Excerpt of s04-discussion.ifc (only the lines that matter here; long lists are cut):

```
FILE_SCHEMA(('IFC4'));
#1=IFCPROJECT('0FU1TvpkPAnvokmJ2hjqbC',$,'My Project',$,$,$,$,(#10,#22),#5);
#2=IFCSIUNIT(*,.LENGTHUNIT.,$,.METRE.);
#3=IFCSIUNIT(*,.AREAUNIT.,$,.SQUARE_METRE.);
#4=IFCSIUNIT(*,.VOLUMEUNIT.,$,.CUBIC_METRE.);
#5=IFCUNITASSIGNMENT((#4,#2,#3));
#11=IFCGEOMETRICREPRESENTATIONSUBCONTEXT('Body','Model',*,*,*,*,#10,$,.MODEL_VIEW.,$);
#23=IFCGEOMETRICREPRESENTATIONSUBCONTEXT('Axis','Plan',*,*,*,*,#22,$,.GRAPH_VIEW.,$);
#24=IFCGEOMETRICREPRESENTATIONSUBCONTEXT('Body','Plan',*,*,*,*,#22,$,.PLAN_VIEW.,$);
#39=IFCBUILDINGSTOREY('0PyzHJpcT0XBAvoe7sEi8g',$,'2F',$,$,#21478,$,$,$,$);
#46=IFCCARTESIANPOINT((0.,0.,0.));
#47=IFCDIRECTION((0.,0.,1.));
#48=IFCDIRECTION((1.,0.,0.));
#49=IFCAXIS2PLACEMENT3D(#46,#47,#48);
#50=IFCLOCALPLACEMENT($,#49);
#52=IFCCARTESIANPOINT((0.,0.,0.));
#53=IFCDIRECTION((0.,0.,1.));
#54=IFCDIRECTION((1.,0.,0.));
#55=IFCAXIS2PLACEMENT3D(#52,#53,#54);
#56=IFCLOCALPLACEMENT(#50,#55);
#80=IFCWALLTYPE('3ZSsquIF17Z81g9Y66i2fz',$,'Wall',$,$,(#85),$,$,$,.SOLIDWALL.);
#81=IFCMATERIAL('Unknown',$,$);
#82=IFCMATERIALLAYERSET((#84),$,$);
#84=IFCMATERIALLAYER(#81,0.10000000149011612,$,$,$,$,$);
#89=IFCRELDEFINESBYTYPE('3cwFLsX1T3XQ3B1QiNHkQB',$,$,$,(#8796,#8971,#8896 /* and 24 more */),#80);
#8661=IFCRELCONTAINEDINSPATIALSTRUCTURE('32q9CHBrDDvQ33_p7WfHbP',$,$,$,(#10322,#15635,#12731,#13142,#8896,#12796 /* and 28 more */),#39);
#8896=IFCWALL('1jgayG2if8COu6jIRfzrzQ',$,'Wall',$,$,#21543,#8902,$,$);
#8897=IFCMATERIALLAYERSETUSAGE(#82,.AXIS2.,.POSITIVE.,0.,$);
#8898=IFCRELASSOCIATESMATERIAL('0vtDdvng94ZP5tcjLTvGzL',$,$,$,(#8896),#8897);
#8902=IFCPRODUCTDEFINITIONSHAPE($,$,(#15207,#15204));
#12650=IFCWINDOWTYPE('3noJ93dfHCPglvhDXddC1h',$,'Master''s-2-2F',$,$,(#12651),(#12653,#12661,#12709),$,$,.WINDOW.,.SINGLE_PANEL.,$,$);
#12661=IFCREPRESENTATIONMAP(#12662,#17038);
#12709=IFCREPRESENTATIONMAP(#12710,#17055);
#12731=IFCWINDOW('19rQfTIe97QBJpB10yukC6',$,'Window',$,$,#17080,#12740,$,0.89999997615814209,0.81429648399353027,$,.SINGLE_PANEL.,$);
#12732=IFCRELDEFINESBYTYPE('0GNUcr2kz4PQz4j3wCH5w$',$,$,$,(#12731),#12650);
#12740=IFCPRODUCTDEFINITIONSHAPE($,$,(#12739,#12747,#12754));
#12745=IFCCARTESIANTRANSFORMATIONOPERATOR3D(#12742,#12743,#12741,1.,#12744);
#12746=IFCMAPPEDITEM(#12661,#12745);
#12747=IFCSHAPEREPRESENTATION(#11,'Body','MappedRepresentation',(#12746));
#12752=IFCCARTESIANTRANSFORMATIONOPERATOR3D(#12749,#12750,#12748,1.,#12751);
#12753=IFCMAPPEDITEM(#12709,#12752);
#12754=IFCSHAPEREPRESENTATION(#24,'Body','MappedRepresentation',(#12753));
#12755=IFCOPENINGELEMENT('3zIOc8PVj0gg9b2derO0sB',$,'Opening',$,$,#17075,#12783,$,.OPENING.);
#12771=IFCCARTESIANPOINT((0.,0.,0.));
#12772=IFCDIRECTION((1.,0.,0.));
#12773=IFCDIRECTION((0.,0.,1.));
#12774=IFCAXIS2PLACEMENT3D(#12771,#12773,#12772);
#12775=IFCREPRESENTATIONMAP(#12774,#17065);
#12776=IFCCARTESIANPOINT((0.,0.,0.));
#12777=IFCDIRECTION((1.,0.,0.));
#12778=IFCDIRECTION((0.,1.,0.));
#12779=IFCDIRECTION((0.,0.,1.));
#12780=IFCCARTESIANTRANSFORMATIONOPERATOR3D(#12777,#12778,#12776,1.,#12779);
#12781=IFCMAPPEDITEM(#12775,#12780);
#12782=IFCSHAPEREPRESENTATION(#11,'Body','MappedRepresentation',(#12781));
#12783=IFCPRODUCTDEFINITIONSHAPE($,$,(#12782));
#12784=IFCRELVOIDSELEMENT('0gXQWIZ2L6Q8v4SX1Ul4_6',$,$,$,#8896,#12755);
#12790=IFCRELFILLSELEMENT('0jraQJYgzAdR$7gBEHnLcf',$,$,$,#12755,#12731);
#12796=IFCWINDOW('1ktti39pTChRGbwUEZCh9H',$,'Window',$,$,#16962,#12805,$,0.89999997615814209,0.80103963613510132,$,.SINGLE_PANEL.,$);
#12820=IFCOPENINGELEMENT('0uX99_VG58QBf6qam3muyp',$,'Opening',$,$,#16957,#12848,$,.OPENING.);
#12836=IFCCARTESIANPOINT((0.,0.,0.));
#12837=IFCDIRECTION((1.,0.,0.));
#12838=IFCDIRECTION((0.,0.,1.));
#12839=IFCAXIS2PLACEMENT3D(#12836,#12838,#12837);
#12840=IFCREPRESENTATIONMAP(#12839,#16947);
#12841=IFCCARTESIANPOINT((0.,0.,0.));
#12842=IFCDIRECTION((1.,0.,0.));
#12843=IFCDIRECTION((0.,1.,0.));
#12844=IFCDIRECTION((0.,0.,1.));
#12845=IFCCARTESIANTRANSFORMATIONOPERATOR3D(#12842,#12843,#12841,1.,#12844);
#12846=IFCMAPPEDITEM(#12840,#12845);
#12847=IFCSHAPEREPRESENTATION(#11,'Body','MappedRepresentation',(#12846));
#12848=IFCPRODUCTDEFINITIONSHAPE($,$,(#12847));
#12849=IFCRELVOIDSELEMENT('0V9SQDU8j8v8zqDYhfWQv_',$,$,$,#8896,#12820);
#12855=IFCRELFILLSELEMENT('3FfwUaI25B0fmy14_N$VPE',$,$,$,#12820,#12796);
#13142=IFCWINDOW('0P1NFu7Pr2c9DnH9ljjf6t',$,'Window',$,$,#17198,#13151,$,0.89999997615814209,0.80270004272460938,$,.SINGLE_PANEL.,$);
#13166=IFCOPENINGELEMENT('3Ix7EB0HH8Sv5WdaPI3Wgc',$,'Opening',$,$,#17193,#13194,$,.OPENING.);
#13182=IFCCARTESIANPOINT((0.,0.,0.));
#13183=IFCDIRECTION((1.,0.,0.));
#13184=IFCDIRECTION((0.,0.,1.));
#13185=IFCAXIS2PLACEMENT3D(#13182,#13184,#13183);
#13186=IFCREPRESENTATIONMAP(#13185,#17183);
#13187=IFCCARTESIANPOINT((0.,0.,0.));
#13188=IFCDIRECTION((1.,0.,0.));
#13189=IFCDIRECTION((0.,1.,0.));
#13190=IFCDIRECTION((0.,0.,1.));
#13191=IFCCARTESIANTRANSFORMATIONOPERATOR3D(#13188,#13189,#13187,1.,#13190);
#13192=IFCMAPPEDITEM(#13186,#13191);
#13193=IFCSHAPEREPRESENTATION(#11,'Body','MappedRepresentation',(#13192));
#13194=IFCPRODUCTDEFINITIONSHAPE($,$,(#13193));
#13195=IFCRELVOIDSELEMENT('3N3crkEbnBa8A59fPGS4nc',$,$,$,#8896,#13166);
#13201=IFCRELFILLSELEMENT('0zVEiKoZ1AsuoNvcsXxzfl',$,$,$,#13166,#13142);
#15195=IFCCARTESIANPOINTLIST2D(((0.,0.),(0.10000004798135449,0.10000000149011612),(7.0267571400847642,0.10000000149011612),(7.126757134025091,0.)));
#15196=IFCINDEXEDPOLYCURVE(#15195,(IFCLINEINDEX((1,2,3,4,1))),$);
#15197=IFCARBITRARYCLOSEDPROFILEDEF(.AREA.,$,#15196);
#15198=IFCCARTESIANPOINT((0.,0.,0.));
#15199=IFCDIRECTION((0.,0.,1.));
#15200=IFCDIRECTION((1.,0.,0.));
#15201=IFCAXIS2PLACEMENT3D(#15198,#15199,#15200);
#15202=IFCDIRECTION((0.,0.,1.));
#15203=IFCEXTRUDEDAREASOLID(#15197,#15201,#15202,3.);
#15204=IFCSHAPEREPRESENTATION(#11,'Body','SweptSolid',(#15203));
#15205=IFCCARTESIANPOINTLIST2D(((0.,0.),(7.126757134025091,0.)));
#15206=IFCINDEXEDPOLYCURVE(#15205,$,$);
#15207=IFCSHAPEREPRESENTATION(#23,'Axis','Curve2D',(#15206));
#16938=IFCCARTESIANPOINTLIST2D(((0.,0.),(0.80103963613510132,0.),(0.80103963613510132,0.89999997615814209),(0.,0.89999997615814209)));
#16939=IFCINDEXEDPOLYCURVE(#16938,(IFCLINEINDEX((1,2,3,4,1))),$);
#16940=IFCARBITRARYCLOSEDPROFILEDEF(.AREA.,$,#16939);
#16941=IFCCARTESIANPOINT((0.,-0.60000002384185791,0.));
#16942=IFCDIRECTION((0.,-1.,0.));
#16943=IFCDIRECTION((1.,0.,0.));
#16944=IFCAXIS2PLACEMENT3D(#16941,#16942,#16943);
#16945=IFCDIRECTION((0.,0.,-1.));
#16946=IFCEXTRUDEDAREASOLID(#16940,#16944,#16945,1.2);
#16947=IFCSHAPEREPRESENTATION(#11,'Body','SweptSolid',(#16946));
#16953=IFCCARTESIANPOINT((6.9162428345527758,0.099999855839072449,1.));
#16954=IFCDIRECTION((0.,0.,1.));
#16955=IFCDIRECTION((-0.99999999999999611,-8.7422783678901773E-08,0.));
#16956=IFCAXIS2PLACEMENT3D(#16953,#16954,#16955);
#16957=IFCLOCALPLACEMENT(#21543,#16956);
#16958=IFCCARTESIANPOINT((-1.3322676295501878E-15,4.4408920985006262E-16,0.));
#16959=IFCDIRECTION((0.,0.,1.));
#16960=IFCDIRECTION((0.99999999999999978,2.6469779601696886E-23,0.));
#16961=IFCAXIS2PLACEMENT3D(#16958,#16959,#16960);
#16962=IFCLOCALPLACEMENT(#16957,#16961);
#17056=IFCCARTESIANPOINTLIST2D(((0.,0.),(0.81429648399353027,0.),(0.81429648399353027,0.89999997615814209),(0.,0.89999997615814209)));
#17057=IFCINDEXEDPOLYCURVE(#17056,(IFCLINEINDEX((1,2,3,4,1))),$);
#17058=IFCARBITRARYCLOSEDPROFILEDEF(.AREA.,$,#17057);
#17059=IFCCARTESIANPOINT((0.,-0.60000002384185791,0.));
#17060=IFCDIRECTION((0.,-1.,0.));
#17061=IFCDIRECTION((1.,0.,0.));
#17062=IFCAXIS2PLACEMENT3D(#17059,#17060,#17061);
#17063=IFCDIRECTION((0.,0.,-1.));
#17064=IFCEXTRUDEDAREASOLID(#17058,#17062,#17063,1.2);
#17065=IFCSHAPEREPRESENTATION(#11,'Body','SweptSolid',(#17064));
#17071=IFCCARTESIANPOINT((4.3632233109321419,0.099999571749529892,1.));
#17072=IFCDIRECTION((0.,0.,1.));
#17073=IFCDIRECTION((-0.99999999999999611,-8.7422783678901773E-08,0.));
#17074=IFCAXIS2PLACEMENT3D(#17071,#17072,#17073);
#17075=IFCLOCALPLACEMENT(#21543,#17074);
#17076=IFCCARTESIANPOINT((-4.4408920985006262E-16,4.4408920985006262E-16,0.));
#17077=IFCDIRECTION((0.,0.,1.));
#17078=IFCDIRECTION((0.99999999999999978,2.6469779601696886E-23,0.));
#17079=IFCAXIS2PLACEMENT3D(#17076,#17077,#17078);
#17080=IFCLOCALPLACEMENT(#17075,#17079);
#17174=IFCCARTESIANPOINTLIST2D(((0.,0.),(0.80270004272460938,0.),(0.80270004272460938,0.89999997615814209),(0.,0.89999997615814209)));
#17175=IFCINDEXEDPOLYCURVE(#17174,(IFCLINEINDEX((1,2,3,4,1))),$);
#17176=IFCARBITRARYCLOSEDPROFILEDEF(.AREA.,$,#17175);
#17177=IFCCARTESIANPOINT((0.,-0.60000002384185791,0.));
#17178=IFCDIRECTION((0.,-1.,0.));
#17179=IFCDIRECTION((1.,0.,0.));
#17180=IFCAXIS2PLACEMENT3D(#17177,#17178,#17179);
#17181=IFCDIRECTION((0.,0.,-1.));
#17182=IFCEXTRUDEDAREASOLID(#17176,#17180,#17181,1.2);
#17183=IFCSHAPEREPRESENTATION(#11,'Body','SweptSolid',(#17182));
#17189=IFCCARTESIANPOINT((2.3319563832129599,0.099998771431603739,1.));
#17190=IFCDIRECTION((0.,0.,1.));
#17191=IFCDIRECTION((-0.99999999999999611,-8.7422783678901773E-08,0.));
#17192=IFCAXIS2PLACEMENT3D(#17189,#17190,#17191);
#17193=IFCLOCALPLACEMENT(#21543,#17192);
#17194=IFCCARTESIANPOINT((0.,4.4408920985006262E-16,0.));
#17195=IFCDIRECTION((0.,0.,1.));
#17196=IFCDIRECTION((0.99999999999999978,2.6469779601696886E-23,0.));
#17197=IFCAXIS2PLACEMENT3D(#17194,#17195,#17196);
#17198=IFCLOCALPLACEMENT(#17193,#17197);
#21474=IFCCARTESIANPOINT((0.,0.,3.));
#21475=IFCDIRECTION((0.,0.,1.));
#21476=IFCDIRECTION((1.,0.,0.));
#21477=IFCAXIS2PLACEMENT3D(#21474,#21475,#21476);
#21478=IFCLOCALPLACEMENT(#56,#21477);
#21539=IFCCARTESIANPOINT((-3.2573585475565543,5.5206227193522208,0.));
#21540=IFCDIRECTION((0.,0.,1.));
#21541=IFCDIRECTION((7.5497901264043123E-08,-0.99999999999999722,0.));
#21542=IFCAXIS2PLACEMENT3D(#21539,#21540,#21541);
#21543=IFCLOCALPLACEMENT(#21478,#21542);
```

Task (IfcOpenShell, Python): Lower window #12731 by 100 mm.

```python
import numpy as np
import ifcopenshell
import ifcopenshell.api.geometry
import ifcopenshell.util.placement
import ifcopenshell.util.unit

model = ifcopenshell.open("s04-discussion.ifc")
unit_scale = ifcopenshell.util.unit.calculate_unit_scale(model)

window = model.by_id(12731)
opening = window.FillsVoids[0].RelatingOpeningElement
dz = -0.1 / unit_scale

shift = np.array([0.0, 0.0, dz])
# The window is placed relative to its opening, so it follows when the opening moves.
matrix = ifcopenshell.util.placement.get_local_placement(opening.ObjectPlacement)
matrix[:3, 3] += shift
ifcopenshell.api.geometry.edit_object_placement(
    model, product=opening, matrix=matrix, is_si=False, should_transform_children=True
)

print(f"moved by {dz * unit_scale:+.3f} m")

model.write("s04-discussion_v2.ifc")
```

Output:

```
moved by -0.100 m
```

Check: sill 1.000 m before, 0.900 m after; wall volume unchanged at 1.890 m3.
